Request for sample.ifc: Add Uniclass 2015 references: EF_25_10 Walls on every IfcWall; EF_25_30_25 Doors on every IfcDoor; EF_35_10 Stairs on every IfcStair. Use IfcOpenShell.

First a look at what the model holds.

```python
import ifcopenshell

model = ifcopenshell.open("sample.ifc")
print(model.schema)
print("classifications:", [c.Name for c in model.by_type("IfcClassification")])
for ifc_class in ("IfcDoor", "IfcRoof", "IfcStair", "IfcWall", "IfcWindow"):
    print(ifc_class, len(model.by_type(ifc_class)))
```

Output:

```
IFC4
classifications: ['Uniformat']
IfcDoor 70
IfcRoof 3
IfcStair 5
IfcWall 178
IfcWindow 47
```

```python
import ifcopenshell
import ifcopenshell.api.classification

model = ifcopenshell.open("sample.ifc")

system = ifcopenshell.api.classification.add_classification(model, classification="Uniclass 2015")

codes = {
    "IfcWall": ("EF_25_10", "Walls"),
    "IfcDoor": ("EF_25_30_25", "Doors"),
    "IfcStair": ("EF_35_10", "Stairs"),
}
for ifc_class, (code, name) in codes.items():
    products = model.by_type(ifc_class)
    ifcopenshell.api.classification.add_reference(
        model, products=products, classification=system, identification=code, name=name
    )
    print(code, len(products))

model.write("sample_v2.ifc")
```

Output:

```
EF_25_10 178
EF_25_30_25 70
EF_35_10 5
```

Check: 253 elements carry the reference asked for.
